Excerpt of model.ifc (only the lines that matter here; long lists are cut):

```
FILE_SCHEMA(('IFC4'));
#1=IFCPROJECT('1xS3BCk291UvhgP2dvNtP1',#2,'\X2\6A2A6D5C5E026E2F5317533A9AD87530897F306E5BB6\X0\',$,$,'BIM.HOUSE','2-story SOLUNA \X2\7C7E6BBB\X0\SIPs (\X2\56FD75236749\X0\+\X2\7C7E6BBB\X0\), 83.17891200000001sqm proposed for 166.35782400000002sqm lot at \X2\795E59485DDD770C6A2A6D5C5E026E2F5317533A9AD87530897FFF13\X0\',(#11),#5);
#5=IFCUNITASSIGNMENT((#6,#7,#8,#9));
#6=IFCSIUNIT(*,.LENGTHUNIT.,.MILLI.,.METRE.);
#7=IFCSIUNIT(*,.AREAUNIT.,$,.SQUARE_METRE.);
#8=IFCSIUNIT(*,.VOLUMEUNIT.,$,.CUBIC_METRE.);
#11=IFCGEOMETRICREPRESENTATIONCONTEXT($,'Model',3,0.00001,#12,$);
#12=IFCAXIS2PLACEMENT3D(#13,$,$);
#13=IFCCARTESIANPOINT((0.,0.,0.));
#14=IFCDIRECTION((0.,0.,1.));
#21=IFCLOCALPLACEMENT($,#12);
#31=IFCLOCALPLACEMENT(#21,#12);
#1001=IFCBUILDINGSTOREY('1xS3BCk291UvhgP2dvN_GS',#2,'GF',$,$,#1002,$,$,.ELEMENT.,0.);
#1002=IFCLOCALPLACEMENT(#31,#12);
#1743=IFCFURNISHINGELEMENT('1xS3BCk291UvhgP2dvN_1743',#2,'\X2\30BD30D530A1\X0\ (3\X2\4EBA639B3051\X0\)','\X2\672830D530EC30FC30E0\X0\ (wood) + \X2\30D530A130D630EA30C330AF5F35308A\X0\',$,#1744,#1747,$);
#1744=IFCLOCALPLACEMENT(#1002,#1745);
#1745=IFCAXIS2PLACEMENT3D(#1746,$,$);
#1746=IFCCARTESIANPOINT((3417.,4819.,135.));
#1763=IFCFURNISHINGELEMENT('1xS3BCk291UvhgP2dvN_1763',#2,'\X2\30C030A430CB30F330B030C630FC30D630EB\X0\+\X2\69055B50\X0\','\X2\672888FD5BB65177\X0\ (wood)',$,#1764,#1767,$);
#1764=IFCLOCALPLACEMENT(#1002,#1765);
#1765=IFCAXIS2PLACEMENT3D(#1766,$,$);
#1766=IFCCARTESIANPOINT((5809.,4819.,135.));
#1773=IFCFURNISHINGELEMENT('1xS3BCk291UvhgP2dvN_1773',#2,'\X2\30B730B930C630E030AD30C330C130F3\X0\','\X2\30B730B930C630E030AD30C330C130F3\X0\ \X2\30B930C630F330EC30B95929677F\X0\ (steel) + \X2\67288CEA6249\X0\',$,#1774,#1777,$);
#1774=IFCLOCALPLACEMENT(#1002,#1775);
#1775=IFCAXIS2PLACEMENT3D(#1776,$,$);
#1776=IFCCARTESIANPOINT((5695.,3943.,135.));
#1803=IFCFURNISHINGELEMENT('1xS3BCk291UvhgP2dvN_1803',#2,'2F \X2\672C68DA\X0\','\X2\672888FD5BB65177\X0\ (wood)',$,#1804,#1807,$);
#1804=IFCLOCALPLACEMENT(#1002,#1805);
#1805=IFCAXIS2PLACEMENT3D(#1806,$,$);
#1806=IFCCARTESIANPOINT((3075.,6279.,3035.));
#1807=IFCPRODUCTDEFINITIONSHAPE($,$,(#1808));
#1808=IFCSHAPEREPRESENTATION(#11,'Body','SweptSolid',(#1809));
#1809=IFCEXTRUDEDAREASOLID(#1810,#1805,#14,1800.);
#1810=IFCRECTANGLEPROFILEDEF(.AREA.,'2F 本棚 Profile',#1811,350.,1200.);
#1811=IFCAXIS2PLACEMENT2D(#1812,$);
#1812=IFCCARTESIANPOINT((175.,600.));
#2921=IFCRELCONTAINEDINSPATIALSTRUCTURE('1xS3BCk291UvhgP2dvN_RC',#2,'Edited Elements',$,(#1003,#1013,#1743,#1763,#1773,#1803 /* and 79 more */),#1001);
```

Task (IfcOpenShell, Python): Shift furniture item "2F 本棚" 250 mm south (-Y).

```python
import ifcopenshell
import ifcopenshell.api.geometry
import ifcopenshell.util.placement

model = ifcopenshell.open("model.ifc")

item = model.by_guid("1xS3BCk291UvhgP2dvN_1803")
matrix = ifcopenshell.util.placement.get_local_placement(item.ObjectPlacement)
matrix[1, 3] -= 250.0
ifcopenshell.api.geometry.edit_object_placement(model, product=item, matrix=matrix, is_si=False)

print(ifcopenshell.util.placement.get_local_placement(item.ObjectPlacement).round(3) + 0.0)

model.write("model_updated.ifc")
```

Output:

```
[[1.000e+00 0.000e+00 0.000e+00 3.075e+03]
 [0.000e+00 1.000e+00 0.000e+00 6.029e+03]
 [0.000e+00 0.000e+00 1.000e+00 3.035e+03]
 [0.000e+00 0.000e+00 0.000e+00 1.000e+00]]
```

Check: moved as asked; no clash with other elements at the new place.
